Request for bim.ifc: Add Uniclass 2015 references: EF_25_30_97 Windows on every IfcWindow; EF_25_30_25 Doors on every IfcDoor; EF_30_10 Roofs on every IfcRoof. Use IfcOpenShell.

First a look at what the model holds.

```python
import ifcopenshell

model = ifcopenshell.open("bim.ifc")
print(model.schema)
print("classifications:", [c.Name for c in model.by_type("IfcClassification")])
for ifc_class in ("IfcDoor", "IfcRoof", "IfcStair", "IfcWall", "IfcWindow"):
    print(ifc_class, len(model.by_type(ifc_class)))
```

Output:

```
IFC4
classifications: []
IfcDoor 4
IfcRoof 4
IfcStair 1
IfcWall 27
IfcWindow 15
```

```python
import ifcopenshell
import ifcopenshell.api.classification

model = ifcopenshell.open("bim.ifc")

system = ifcopenshell.api.classification.add_classification(model, classification="Uniclass 2015")

codes = {
    "IfcWindow": ("EF_25_30_97", "Windows"),
    "IfcDoor": ("EF_25_30_25", "Doors"),
    "IfcRoof": ("EF_30_10", "Roofs"),
}
for ifc_class, (code, name) in codes.items():
    products = model.by_type(ifc_class)
    ifcopenshell.api.classification.add_reference(
        model, products=products, classification=system, identification=code, name=name
    )
    print(code, len(products))

model.write("bim_edited.ifc")
```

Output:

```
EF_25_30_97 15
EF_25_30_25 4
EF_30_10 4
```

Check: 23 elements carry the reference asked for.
